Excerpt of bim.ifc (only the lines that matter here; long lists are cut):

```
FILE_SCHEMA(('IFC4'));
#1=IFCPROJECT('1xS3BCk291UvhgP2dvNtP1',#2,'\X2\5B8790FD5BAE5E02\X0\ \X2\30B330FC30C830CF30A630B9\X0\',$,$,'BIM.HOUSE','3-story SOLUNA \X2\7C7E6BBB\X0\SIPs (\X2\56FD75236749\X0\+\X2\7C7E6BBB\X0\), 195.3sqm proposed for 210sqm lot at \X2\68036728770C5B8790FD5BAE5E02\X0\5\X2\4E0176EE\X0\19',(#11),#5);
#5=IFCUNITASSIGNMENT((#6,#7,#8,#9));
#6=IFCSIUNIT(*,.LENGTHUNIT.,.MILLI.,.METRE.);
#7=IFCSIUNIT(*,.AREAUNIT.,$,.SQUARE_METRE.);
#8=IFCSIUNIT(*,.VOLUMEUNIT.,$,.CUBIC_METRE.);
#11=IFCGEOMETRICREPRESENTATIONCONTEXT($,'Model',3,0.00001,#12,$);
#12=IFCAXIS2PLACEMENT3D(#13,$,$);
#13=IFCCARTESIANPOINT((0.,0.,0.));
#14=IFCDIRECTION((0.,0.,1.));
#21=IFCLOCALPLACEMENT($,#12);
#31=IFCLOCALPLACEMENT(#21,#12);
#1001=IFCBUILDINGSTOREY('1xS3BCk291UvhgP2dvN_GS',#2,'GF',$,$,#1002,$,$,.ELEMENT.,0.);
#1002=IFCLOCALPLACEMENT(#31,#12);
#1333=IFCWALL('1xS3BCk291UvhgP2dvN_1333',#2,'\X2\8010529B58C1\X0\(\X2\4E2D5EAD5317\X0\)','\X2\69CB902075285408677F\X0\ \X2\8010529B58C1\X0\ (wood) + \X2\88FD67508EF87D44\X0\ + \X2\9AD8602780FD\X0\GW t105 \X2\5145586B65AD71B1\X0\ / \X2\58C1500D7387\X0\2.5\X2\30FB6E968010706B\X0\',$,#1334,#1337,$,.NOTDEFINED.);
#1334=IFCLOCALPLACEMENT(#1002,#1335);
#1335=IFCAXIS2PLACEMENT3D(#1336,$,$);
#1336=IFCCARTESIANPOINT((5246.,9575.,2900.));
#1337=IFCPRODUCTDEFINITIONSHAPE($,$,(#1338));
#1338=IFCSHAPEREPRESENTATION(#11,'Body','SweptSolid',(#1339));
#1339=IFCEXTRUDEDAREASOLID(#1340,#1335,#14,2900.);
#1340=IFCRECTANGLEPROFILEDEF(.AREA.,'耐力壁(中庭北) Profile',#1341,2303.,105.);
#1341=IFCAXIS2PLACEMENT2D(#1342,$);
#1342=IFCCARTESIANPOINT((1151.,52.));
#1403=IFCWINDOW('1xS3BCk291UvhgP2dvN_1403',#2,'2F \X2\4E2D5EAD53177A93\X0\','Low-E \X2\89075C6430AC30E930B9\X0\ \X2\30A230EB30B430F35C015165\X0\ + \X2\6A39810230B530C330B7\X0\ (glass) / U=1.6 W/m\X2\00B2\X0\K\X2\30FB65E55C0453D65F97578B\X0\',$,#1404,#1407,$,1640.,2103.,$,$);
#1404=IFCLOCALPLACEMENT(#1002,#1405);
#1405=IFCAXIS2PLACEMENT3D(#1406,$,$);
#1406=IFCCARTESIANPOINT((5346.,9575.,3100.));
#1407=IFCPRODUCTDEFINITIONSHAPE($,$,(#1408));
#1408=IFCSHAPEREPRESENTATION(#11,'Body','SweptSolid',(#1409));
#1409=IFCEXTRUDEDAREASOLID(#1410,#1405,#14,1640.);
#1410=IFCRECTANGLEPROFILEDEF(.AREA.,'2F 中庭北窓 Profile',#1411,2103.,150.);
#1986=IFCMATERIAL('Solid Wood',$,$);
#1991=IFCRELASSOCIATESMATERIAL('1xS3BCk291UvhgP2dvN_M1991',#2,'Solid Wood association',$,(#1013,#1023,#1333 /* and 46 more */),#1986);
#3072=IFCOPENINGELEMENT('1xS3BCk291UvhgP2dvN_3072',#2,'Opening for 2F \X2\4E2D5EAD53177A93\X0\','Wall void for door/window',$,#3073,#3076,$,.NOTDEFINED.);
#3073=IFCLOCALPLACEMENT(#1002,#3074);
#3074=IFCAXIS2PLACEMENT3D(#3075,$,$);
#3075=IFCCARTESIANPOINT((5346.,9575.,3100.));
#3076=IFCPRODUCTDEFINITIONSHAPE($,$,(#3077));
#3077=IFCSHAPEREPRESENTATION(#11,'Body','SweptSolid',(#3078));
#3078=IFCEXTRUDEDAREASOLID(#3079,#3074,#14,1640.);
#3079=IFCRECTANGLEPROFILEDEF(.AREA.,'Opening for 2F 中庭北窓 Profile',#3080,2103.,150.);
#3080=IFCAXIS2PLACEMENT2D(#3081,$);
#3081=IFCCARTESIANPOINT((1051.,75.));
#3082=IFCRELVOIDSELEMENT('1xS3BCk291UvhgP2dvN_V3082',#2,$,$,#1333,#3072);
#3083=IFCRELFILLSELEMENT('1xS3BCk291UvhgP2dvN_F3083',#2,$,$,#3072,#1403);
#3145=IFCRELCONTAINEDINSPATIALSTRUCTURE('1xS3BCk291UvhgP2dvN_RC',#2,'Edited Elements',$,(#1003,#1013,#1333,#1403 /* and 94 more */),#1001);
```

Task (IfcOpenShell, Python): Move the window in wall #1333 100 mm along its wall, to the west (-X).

```python
import ifcopenshell
import ifcopenshell.api.geometry
import ifcopenshell.util.placement

model = ifcopenshell.open("bim.ifc")

window = model.by_guid("1xS3BCk291UvhgP2dvN_1403")
opening = window.FillsVoids[0].RelatingOpeningElement
wall = opening.VoidsElements[0].RelatingBuildingElement

wall_matrix = ifcopenshell.util.placement.get_local_placement(wall.ObjectPlacement)
shift = wall_matrix[:3, 0] * -100.0
before = ifcopenshell.util.placement.get_local_placement(window.ObjectPlacement)[:3, 3].copy()

# The window is not placed relative to its opening, so move both.
for product in (opening, window):
    matrix = ifcopenshell.util.placement.get_local_placement(product.ObjectPlacement)
    matrix[:3, 3] += shift
    ifcopenshell.api.geometry.edit_object_placement(model, product=product, matrix=matrix, is_si=False)

after = ifcopenshell.util.placement.get_local_placement(window.ObjectPlacement)[:3, 3]
print("window moved by", (after - before).round(3) + 0.0)

model.write("bim_rev.ifc")
```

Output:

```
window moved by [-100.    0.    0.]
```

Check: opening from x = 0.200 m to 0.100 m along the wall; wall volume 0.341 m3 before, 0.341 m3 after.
